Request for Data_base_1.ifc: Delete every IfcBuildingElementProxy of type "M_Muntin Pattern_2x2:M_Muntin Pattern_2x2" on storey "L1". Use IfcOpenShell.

First a look at what the model holds.

```python
import ifcopenshell
import ifcopenshell.util.element

model = ifcopenshell.open("Data_base_1.ifc")
print(model.schema)
storey = next(s for s in model.by_type("IfcBuildingStorey") if s.Name == "L1")
proxies = [e for e in ifcopenshell.util.element.get_decomposition(storey) if e.is_a("IfcBuildingElementProxy")]
seen = {}
for e in proxies:
    element_type = ifcopenshell.util.element.get_type(e)
    name = element_type.Name if element_type not in (None, e) else None
    seen[name] = seen.get(name, 0) + 1
for name, count in sorted(seen.items(), key=str):
    print(count, "x", name)
```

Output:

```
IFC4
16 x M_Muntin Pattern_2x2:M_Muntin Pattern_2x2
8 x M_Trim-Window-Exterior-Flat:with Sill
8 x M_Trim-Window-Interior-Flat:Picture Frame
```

```python
import ifcopenshell
import ifcopenshell.api.root
import ifcopenshell.util.element

model = ifcopenshell.open("Data_base_1.ifc")

storey = next(s for s in model.by_type("IfcBuildingStorey") if s.Name == "L1")
proxies = [e for e in ifcopenshell.util.element.get_decomposition(storey) if e.is_a("IfcBuildingElementProxy")]
targets = [e for e in proxies if (t := ifcopenshell.util.element.get_type(e)) not in (None, e) and t.Name == "M_Muntin Pattern_2x2:M_Muntin Pattern_2x2"]

for e in targets:
    ifcopenshell.api.root.remove_product(model, product=e)
print(len(targets), "removed")

model.write("Data_base_1_v2.ifc")
```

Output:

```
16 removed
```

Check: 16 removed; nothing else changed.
